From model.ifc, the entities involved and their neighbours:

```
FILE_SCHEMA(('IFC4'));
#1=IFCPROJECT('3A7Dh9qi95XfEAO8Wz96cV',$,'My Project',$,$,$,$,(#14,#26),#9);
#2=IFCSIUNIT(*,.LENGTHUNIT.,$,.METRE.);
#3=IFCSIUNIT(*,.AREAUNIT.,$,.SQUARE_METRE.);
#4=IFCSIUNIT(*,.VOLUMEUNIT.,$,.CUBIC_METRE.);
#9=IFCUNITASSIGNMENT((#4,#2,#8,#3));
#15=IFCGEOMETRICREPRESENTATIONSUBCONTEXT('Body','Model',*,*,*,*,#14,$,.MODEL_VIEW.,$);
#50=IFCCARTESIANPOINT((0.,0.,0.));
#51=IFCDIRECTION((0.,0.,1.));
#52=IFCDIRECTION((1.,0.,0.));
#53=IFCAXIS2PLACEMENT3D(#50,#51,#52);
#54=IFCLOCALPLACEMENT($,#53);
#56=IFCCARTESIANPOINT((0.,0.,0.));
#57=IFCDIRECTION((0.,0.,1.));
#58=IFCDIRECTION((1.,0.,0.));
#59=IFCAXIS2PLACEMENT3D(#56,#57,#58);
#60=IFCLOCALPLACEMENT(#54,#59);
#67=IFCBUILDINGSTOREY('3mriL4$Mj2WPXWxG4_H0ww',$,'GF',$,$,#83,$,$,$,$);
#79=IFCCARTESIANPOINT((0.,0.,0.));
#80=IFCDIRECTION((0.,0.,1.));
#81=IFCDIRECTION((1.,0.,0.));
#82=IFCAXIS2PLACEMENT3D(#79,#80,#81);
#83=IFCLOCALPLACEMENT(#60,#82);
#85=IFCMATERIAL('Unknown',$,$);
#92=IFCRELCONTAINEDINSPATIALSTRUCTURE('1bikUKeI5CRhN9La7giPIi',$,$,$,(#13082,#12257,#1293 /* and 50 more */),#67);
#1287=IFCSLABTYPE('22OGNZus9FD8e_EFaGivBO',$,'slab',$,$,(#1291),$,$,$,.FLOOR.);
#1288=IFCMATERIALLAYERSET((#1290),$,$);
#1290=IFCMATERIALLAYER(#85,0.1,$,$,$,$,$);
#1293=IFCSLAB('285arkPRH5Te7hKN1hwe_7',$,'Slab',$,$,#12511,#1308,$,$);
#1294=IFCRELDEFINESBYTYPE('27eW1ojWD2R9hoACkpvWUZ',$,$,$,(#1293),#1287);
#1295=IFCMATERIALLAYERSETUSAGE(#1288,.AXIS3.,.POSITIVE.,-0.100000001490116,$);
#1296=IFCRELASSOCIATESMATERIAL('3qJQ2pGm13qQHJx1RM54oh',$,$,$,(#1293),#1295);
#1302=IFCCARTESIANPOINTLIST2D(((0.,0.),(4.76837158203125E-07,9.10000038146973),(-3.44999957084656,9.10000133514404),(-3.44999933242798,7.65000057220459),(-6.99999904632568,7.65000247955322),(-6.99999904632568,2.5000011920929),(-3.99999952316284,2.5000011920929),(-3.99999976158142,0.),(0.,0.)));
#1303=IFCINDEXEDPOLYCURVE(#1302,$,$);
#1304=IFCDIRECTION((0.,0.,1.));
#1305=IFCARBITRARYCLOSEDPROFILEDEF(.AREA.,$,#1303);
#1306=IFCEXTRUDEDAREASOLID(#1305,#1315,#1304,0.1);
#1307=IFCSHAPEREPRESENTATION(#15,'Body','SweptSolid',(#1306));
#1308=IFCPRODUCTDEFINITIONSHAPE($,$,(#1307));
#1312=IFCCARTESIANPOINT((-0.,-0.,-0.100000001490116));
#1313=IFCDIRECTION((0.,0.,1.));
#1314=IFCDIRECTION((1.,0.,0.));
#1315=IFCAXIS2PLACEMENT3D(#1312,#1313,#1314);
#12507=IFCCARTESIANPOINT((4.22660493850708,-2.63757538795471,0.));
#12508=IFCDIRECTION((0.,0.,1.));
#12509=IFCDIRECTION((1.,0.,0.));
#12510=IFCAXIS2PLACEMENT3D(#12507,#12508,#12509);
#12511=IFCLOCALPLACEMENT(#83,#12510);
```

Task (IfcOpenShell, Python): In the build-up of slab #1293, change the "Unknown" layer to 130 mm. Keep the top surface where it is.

```python
import ifcopenshell
import ifcopenshell.util.element
import ifcopenshell.util.representation

model = ifcopenshell.open("model.ifc")

layer_set = model.by_id(1288)
layer = next(l for l in layer_set.MaterialLayers if l.Material and l.Material.Name == "Unknown")
change = 0.13 - layer.LayerThickness
layer.LayerThickness += change

# Geometry does not follow the layer set by itself.
slabs = [e for e in ifcopenshell.util.element.get_elements_by_material(model, layer_set) if e.is_a("IfcSlab")]
for slab in sorted(slabs, key=lambda e: e.id()):
    body = ifcopenshell.util.representation.get_representation(slab, "Model", "Body")
    solid = body.Items[0]
    old_depth = solid.Depth
    solid.Depth += change
    # Extruded upwards: lower the start of the extrusion so the top stays.
    x, y, z = solid.Position.Location.Coordinates
    solid.Position.Location = model.createIfcCartesianPoint((x, y, z - change))
    print(slab.id(), f"{old_depth:g} -> {solid.Depth:g}")

# The layers are counted up from the underside, which has moved.
for usage in {ifcopenshell.util.element.get_material(slab) for slab in slabs}:
    usage.OffsetFromReferenceLine -= change

model.write("model_edited.ifc")
```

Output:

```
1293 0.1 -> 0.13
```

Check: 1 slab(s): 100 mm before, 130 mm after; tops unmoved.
